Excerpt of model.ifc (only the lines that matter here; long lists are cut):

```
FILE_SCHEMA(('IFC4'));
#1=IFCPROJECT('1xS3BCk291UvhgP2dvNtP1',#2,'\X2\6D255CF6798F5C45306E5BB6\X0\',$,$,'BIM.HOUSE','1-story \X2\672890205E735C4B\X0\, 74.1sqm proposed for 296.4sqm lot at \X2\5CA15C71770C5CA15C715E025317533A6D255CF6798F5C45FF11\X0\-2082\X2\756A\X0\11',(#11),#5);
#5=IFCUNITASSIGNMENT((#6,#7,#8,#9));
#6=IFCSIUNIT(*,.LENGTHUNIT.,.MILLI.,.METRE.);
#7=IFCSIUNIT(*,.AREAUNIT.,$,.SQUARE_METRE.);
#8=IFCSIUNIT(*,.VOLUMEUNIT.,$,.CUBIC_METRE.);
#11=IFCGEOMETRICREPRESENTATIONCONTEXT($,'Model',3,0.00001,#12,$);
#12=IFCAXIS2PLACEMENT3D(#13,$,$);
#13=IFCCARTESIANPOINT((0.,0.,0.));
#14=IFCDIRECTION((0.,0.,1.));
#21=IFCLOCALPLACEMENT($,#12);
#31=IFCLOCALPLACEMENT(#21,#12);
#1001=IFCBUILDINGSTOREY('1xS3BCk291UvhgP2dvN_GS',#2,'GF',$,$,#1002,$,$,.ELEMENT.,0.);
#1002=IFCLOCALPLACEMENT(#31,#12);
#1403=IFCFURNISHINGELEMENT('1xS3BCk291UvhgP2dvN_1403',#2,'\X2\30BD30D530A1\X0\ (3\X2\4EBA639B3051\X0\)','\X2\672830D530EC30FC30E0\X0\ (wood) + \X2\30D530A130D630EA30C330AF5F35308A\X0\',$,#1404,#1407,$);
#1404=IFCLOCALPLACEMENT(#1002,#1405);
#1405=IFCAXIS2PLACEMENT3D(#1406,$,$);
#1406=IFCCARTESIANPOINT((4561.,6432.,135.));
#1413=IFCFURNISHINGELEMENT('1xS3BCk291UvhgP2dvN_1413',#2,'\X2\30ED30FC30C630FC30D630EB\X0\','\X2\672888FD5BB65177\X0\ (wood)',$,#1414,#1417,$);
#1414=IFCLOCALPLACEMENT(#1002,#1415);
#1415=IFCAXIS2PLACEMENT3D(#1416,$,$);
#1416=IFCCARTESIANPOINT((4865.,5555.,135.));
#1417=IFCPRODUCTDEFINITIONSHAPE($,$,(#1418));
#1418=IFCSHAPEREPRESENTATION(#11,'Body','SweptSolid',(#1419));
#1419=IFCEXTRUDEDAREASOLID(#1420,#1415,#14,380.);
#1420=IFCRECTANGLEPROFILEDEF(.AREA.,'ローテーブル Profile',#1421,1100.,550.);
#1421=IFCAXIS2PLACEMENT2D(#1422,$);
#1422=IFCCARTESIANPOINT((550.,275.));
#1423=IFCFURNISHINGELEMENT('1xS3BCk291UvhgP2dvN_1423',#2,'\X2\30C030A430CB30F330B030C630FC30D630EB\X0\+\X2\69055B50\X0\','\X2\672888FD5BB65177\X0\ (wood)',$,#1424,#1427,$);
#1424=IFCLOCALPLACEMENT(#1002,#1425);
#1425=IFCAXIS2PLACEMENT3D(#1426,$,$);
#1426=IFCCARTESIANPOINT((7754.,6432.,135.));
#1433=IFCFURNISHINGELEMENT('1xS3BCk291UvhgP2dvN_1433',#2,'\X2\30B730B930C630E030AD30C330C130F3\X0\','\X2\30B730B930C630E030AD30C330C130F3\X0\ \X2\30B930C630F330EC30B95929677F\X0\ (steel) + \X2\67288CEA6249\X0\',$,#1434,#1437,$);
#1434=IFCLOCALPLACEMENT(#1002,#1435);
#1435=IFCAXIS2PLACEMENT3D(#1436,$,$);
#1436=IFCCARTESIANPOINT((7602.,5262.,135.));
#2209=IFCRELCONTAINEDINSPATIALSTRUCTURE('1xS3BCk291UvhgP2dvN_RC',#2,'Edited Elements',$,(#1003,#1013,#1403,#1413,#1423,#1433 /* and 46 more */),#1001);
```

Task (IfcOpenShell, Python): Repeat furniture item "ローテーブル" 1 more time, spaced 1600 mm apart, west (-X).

```python
import numpy as np
import ifcopenshell
import ifcopenshell.api.geometry
import ifcopenshell.api.root
import ifcopenshell.util.element
import ifcopenshell.util.placement

model = ifcopenshell.open("model.ifc")


def reuse_history(source, copy):
    """copy_class also copies each property set's owner history, people and application; keep the originals."""
    for rel in copy.IsDefinedBy:
        if rel.is_a("IfcRelDefinesByProperties") and (history := rel.RelatingPropertyDefinition.OwnerHistory):
            rel.RelatingPropertyDefinition.OwnerHistory = source.OwnerHistory
            ifcopenshell.util.element.remove_deep2(model, history)


source = model.by_guid("1xS3BCk291UvhgP2dvN_1413")
base = ifcopenshell.util.placement.get_local_placement(source.ObjectPlacement)
step = np.array([-1.0, 0.0, 0.0]) * 1600.0

for i in range(1, 2):
    copy = ifcopenshell.api.root.copy_class(model, product=source)
    copy.Representation = ifcopenshell.util.element.copy_deep(
        model, source.Representation, exclude=["IfcGeometricRepresentationContext", "IfcRepresentationMap"]
    )
    reuse_history(source, copy)
    matrix = base.copy()
    matrix[:3, 3] += i * step
    print("added at", matrix[:3, 3].round(3) + 0.0)
    ifcopenshell.api.geometry.edit_object_placement(model, product=copy, matrix=matrix, is_si=False)

model.write("model_updated.ifc")
```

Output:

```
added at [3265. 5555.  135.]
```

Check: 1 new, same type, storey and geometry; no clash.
